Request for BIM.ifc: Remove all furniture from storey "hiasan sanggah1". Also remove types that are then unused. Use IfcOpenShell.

First a look at what the model holds.

```python
import ifcopenshell
import ifcopenshell.util.element

model = ifcopenshell.open("BIM.ifc")
print(model.schema)
storey = next(s for s in model.by_type("IfcBuildingStorey") if s.Name == "hiasan sanggah1")
furniture = [e for e in ifcopenshell.util.element.get_decomposition(storey) if e.is_a("IfcFurnishingElement")]
seen = {}
for e in furniture:
    element_type = ifcopenshell.util.element.get_type(e)
    name = element_type.Name if element_type not in (None, e) else None
    seen[name] = seen.get(name, 0) + 1
for name, count in sorted(seen.items(), key=str):
    print(count, "x", name)
```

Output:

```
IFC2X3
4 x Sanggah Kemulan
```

```python
import ifcopenshell
import ifcopenshell.api.root
import ifcopenshell.util.element

model = ifcopenshell.open("BIM.ifc")

storey = next(s for s in model.by_type("IfcBuildingStorey") if s.Name == "hiasan sanggah1")
furniture = [e for e in ifcopenshell.util.element.get_decomposition(storey) if e.is_a("IfcFurnishingElement")]
types = {ifcopenshell.util.element.get_type(e) for e in furniture} - {None, *furniture}

for e in furniture:
    ifcopenshell.api.root.remove_product(model, product=e)
print(len(furniture), "removed")

unused = [t for t in types if not ifcopenshell.util.element.get_types(t)]
for t in unused:
    ifcopenshell.api.root.remove_product(model, product=t)
print(len(unused), "unused types removed")

model.write("BIM_rev.ifc")
```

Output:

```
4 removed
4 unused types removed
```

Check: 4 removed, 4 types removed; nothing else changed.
